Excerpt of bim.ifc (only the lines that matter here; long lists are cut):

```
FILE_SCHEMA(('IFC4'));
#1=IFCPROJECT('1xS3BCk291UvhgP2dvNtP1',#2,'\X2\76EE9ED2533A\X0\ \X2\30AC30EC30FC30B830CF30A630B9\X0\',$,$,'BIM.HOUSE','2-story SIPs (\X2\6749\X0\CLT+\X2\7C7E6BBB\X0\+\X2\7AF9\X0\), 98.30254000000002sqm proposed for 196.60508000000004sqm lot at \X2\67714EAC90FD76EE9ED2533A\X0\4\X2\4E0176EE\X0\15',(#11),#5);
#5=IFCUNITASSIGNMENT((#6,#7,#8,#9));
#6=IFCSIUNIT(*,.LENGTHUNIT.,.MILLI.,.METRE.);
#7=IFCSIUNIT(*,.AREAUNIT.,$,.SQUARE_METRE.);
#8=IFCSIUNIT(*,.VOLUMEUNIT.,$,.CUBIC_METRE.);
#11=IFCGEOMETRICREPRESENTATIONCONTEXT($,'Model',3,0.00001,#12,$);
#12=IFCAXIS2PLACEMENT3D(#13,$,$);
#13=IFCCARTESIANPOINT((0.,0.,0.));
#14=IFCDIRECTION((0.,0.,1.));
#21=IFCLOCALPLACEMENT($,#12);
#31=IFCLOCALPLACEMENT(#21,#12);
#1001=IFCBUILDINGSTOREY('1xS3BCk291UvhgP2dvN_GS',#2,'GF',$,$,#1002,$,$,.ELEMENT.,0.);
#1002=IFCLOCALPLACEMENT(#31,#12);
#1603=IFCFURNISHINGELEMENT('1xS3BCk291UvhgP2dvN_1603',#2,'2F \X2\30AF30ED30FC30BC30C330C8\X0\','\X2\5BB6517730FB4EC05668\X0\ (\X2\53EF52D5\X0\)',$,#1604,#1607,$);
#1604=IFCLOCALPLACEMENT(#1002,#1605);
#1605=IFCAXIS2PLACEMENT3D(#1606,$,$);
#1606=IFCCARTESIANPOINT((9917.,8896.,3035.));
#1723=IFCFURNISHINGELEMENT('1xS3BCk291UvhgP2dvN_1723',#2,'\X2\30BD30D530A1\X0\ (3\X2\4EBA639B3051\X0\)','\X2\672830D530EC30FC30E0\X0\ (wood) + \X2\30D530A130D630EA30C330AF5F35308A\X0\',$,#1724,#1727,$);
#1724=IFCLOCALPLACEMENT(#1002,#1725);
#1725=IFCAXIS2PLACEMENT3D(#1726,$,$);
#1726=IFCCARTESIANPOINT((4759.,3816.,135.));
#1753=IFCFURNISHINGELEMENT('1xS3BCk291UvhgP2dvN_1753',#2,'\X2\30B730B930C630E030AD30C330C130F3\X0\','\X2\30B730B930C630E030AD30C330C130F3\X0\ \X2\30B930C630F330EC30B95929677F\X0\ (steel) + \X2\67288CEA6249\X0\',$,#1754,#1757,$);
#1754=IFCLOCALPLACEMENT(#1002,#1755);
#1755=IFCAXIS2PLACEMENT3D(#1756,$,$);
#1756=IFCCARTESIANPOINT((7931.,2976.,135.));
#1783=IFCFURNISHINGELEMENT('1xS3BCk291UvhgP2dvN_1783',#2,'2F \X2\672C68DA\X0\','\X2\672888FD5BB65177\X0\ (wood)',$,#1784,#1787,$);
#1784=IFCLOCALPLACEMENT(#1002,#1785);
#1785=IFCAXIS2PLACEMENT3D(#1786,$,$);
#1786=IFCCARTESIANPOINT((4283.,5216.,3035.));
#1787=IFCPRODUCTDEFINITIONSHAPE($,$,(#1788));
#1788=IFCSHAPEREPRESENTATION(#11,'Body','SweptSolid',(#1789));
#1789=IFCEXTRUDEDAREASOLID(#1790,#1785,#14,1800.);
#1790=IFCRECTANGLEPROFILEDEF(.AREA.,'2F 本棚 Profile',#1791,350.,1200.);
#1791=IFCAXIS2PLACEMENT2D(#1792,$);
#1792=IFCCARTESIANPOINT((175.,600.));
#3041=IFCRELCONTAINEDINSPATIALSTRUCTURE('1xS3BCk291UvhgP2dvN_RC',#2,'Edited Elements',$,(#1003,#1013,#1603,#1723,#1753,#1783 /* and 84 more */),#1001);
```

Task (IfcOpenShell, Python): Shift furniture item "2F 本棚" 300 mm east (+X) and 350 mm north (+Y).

```python
import ifcopenshell
import ifcopenshell.api.geometry
import ifcopenshell.util.placement
import ifcopenshell.util.unit

model = ifcopenshell.open("bim.ifc")
unit_scale = ifcopenshell.util.unit.calculate_unit_scale(model)

item = model.by_guid("1xS3BCk291UvhgP2dvN_1783")
matrix = ifcopenshell.util.placement.get_local_placement(item.ObjectPlacement)
matrix[0, 3] += 0.3 / unit_scale
matrix[1, 3] += 0.35 / unit_scale
ifcopenshell.api.geometry.edit_object_placement(model, product=item, matrix=matrix, is_si=False)

print(ifcopenshell.util.placement.get_local_placement(item.ObjectPlacement).round(3) + 0.0)

model.write("bim_updated.ifc")
```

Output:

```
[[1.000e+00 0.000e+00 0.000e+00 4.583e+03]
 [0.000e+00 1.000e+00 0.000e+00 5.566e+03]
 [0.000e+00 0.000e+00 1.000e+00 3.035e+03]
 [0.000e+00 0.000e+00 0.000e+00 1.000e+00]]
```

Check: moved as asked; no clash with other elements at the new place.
